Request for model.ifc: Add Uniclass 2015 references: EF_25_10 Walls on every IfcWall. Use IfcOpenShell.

First a look at what the model holds.

```python
import ifcopenshell

model = ifcopenshell.open("model.ifc")
print(model.schema)
print("classifications:", [c.Name for c in model.by_type("IfcClassification")])
for ifc_class in ("IfcDoor", "IfcRoof", "IfcStair", "IfcWall", "IfcWindow"):
    print(ifc_class, len(model.by_type(ifc_class)))
```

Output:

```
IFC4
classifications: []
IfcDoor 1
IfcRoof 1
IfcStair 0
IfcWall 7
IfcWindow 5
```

```python
import ifcopenshell
import ifcopenshell.api.classification

model = ifcopenshell.open("model.ifc")

system = ifcopenshell.api.classification.add_classification(model, classification="Uniclass 2015")

codes = {
    "IfcWall": ("EF_25_10", "Walls"),
}
for ifc_class, (code, name) in codes.items():
    products = model.by_type(ifc_class)
    ifcopenshell.api.classification.add_reference(
        model, products=products, classification=system, identification=code, name=name
    )
    print(code, len(products))

model.write("model_rev.ifc")
```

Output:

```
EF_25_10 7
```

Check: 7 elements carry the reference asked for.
